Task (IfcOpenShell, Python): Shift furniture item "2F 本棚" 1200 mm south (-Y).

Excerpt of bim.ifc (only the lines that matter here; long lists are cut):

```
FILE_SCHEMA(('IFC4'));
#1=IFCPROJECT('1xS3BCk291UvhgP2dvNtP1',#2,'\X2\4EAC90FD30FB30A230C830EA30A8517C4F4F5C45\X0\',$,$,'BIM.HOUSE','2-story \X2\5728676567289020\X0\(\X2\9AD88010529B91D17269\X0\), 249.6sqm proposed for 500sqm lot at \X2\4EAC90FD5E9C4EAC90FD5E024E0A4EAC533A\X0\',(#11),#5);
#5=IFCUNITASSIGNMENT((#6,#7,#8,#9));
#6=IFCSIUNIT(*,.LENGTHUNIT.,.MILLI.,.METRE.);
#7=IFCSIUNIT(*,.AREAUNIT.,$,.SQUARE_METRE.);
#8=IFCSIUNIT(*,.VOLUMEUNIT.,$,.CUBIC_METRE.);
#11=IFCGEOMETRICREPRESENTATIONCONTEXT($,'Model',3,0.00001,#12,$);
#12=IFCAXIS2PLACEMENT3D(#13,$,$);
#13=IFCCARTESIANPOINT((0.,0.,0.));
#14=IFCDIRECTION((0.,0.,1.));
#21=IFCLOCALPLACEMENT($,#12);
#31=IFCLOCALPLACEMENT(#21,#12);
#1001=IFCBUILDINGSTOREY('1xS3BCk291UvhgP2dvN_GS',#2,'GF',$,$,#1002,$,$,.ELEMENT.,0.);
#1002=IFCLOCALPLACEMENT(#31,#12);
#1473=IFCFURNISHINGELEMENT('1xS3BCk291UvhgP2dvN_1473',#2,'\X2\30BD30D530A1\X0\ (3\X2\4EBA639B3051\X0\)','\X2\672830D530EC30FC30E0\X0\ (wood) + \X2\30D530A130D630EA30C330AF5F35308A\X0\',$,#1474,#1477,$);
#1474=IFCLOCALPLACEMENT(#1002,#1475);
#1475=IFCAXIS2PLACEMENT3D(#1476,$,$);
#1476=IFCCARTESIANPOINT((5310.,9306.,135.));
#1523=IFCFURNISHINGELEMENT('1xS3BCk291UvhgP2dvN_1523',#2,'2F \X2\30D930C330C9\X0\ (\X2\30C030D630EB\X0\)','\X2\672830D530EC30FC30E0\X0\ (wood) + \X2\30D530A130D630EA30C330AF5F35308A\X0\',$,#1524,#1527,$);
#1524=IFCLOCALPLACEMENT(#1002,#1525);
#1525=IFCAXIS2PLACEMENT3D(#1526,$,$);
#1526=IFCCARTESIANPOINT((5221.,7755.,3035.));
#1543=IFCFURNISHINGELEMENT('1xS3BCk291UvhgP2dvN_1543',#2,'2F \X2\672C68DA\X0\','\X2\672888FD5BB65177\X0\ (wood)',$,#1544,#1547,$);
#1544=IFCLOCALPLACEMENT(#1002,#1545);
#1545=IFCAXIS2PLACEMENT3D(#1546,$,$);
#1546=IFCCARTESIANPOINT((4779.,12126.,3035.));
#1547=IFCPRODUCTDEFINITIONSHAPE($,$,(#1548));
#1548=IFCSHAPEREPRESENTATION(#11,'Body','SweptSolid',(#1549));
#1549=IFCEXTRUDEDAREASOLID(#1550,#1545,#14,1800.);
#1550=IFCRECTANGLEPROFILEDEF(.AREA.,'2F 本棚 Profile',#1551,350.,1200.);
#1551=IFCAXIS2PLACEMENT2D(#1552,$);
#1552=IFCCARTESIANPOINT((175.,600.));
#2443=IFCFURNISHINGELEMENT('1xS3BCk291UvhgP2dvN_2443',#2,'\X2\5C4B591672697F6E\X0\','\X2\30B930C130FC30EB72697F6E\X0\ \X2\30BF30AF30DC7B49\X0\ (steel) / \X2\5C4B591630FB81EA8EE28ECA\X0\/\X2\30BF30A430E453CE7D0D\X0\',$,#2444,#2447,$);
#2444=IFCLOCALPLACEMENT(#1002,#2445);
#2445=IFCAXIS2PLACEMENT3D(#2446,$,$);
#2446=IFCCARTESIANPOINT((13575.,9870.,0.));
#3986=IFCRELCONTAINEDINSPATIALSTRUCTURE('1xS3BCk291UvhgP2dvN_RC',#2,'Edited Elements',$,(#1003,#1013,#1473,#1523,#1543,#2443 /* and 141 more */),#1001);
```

```python
import ifcopenshell
import ifcopenshell.api.geometry
import ifcopenshell.util.placement
import ifcopenshell.util.unit

model = ifcopenshell.open("bim.ifc")
unit_scale = ifcopenshell.util.unit.calculate_unit_scale(model)

item = model.by_id(1543)
matrix = ifcopenshell.util.placement.get_local_placement(item.ObjectPlacement)
matrix[1, 3] -= 1.2 / unit_scale
ifcopenshell.api.geometry.edit_object_placement(model, product=item, matrix=matrix, is_si=False)

print(ifcopenshell.util.placement.get_local_placement(item.ObjectPlacement).round(3) + 0.0)

model.write("bim_updated.ifc")
```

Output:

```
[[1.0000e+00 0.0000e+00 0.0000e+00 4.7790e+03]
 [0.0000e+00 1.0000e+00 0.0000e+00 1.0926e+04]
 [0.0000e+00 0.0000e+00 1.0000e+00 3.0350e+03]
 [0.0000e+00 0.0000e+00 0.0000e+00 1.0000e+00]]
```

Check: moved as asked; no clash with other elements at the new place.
